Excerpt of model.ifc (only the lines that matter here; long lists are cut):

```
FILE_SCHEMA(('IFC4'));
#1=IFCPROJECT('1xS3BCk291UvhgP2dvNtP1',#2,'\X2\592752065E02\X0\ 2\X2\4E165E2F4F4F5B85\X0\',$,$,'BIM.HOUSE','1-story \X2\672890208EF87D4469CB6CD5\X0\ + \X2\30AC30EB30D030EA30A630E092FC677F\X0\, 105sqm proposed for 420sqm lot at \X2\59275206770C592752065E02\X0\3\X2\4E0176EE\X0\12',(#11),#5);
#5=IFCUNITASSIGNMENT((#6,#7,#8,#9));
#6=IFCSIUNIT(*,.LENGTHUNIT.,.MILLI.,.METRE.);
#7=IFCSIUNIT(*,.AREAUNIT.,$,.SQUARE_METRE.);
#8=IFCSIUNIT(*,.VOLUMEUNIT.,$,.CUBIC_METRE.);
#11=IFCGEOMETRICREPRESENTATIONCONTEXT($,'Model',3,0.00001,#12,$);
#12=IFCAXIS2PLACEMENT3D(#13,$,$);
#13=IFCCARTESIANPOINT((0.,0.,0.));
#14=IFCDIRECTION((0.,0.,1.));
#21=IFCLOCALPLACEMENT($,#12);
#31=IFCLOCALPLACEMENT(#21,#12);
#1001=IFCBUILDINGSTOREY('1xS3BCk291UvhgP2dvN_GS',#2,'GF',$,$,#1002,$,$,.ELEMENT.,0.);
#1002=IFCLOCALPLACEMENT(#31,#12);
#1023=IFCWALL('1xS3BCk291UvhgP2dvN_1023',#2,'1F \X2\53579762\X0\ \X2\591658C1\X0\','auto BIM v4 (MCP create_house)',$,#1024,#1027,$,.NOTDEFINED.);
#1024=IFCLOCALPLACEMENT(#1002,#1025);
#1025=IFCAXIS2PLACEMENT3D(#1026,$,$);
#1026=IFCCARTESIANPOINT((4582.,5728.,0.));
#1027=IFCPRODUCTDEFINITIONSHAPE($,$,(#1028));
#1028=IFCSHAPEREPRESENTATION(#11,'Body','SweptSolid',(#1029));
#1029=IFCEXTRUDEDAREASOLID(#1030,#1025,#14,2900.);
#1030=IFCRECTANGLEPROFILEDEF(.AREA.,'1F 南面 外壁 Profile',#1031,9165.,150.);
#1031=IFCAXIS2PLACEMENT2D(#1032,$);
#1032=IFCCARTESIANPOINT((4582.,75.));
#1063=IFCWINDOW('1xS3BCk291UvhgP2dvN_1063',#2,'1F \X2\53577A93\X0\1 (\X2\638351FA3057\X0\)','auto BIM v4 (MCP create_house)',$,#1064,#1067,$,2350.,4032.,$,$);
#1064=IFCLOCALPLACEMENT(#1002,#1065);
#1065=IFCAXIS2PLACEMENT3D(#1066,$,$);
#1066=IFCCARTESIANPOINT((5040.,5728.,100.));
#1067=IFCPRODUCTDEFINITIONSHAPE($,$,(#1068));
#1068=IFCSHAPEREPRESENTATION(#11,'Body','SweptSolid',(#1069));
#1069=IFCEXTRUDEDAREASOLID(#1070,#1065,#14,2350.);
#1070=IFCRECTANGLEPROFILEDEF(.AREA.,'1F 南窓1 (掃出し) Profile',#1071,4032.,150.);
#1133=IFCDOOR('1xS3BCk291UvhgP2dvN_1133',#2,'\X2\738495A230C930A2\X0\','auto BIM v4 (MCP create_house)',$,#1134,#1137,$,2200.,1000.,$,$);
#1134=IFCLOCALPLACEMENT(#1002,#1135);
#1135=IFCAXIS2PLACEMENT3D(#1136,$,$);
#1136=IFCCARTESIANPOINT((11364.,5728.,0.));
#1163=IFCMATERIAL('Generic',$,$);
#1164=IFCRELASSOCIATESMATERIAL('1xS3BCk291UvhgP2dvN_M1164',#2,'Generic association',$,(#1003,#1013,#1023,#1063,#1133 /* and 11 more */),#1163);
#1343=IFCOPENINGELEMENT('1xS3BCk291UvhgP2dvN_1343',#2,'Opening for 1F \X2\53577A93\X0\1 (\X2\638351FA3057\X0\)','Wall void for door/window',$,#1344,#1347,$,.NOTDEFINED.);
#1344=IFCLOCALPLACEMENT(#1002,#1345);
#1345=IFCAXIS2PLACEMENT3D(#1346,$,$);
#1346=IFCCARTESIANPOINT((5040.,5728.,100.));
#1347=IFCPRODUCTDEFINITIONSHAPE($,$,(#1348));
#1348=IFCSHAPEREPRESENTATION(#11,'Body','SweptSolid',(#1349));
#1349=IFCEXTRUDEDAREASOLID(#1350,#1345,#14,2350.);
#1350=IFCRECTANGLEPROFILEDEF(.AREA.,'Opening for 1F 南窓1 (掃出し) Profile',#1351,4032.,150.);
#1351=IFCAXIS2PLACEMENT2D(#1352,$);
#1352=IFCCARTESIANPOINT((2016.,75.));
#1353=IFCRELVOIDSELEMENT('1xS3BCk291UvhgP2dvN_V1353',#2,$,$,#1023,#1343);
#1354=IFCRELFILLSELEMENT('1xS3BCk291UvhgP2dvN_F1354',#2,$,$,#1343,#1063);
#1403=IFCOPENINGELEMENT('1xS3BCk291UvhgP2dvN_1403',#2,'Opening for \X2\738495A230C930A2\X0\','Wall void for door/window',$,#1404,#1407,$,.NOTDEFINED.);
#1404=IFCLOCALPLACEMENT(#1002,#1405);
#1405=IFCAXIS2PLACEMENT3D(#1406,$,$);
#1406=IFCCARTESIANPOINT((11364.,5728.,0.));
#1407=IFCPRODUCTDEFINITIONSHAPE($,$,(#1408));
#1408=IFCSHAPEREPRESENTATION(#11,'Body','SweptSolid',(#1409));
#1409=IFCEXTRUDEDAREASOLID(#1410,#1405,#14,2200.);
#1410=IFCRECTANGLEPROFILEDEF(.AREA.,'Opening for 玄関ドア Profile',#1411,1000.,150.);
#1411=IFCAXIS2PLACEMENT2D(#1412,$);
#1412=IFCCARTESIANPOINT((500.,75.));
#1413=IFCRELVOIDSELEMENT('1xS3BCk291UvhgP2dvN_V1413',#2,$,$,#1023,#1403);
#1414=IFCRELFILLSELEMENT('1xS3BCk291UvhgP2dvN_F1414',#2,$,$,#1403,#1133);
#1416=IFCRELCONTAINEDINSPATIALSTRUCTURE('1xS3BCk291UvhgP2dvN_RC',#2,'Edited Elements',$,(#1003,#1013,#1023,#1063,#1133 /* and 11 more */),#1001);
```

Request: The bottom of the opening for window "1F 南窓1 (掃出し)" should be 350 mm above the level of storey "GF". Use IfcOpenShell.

```python
import numpy as np
import ifcopenshell
import ifcopenshell.api.geometry
import ifcopenshell.geom
import ifcopenshell.util.element
import ifcopenshell.util.placement
import ifcopenshell.util.shape
import ifcopenshell.util.unit

model = ifcopenshell.open("model.ifc")
unit_scale = ifcopenshell.util.unit.calculate_unit_scale(model)

window = model.by_guid("1xS3BCk291UvhgP2dvN_1063")
opening = window.FillsVoids[0].RelatingOpeningElement
storey = ifcopenshell.util.element.get_container(window, ifc_class="IfcBuildingStorey")
level = ifcopenshell.util.placement.get_local_placement(storey.ObjectPlacement)[2, 3]

# The opening's origin need not be at the sill, so measure its lowest point.
shape = ifcopenshell.geom.create_shape(ifcopenshell.geom.settings(), opening)
bottom = ifcopenshell.util.shape.get_shape_bottom_elevation(shape, shape.geometry) / unit_scale
dz = level + 350.0 - bottom

shift = np.array([0.0, 0.0, dz])
# The window is not placed relative to its opening, so move both.
for product in (opening, window):
    matrix = ifcopenshell.util.placement.get_local_placement(product.ObjectPlacement)
    matrix[:3, 3] += shift
    ifcopenshell.api.geometry.edit_object_placement(model, product=product, matrix=matrix, is_si=False)

print(f"moved by {dz * unit_scale:+.3f} m")

model.write("model_v2.ifc")
```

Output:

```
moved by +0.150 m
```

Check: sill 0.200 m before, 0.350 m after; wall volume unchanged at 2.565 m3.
